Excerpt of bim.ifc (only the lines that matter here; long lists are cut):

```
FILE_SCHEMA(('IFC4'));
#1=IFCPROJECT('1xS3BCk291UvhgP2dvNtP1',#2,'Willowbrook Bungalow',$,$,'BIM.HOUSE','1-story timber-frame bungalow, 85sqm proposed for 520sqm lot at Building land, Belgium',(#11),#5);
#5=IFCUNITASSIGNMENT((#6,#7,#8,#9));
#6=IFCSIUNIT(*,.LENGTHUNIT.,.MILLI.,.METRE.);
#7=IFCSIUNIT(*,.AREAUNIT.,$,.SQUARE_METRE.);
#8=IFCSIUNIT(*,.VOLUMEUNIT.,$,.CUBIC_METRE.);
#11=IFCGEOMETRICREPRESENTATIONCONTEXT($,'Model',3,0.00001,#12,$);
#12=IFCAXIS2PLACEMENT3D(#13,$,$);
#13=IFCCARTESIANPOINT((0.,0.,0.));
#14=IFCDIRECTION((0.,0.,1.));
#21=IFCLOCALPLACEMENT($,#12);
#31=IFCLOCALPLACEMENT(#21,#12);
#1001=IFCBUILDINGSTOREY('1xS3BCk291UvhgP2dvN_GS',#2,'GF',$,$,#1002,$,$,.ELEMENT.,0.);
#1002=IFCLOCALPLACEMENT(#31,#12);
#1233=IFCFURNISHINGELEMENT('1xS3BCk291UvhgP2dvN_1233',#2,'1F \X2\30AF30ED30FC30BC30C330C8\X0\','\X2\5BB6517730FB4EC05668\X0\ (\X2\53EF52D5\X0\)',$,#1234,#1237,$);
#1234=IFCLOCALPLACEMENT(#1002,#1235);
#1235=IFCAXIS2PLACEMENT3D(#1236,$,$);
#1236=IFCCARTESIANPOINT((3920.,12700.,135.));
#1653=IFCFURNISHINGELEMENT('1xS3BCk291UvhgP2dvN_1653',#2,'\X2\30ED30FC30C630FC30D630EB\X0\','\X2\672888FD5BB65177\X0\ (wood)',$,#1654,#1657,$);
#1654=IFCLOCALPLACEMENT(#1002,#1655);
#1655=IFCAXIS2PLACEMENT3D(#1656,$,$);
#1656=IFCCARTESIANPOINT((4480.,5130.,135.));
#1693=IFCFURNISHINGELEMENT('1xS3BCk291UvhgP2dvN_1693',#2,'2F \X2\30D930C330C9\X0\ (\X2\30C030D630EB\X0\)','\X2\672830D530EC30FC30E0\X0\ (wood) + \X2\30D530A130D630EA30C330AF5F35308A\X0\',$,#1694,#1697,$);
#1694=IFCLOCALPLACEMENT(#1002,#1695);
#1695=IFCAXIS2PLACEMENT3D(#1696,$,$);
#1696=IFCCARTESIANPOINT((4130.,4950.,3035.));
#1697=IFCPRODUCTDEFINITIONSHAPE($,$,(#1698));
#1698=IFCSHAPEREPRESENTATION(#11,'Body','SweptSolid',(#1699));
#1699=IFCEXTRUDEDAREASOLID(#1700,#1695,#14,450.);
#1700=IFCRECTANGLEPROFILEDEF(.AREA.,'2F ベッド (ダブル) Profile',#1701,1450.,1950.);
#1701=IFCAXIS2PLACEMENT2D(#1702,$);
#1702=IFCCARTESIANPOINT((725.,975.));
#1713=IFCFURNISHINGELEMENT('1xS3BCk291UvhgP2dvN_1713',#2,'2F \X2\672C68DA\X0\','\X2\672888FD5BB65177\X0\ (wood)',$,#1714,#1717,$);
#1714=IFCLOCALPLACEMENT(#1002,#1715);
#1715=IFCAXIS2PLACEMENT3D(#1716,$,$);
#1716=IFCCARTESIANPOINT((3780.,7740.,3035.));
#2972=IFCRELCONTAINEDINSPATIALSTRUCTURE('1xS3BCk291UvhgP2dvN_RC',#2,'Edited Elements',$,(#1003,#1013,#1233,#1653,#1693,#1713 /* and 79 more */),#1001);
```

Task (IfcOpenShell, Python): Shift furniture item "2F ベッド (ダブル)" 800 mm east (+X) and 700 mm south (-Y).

```python
import ifcopenshell
import ifcopenshell.api.geometry
import ifcopenshell.util.placement
import ifcopenshell.util.unit

model = ifcopenshell.open("bim.ifc")
unit_scale = ifcopenshell.util.unit.calculate_unit_scale(model)

item = model.by_guid("1xS3BCk291UvhgP2dvN_1693")
matrix = ifcopenshell.util.placement.get_local_placement(item.ObjectPlacement)
matrix[0, 3] += 0.8 / unit_scale
matrix[1, 3] -= 0.7 / unit_scale
ifcopenshell.api.geometry.edit_object_placement(model, product=item, matrix=matrix, is_si=False)

print(ifcopenshell.util.placement.get_local_placement(item.ObjectPlacement).round(3) + 0.0)

model.write("bim_edited.ifc")
```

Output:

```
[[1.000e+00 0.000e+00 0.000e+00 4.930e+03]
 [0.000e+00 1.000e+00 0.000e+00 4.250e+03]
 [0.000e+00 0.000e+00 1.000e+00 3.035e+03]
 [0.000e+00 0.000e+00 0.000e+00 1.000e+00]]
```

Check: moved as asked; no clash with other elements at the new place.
